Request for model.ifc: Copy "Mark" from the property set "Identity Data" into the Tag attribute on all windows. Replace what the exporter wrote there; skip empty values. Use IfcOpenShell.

First a look at what the model holds.

```python
import ifcopenshell
import ifcopenshell.util.element

model = ifcopenshell.open("model.ifc")
print(model.schema)
windows = model.by_type("IfcWindow")
print(len(windows), "windows")
for e in windows[:8]:
    source = ifcopenshell.util.element.get_pset(e, "Identity Data", "Mark")
    target = e.Tag
    print(e.id(), repr(source), repr(target), sep=" | ")
```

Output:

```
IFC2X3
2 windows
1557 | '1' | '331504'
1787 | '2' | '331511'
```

```python
import ifcopenshell
import ifcopenshell.util.element

model = ifcopenshell.open("model.ifc")

count = 0
for e in model.by_type("IfcWindow"):
    value = ifcopenshell.util.element.get_pset(e, "Identity Data", "Mark")
    current = e.Tag
    if not value or not value.strip() or current == value:
        continue
    e.Tag = value
    count += 1

print(count, "windows updated")

model.write("model_updated.ifc")
```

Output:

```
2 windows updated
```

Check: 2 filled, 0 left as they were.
